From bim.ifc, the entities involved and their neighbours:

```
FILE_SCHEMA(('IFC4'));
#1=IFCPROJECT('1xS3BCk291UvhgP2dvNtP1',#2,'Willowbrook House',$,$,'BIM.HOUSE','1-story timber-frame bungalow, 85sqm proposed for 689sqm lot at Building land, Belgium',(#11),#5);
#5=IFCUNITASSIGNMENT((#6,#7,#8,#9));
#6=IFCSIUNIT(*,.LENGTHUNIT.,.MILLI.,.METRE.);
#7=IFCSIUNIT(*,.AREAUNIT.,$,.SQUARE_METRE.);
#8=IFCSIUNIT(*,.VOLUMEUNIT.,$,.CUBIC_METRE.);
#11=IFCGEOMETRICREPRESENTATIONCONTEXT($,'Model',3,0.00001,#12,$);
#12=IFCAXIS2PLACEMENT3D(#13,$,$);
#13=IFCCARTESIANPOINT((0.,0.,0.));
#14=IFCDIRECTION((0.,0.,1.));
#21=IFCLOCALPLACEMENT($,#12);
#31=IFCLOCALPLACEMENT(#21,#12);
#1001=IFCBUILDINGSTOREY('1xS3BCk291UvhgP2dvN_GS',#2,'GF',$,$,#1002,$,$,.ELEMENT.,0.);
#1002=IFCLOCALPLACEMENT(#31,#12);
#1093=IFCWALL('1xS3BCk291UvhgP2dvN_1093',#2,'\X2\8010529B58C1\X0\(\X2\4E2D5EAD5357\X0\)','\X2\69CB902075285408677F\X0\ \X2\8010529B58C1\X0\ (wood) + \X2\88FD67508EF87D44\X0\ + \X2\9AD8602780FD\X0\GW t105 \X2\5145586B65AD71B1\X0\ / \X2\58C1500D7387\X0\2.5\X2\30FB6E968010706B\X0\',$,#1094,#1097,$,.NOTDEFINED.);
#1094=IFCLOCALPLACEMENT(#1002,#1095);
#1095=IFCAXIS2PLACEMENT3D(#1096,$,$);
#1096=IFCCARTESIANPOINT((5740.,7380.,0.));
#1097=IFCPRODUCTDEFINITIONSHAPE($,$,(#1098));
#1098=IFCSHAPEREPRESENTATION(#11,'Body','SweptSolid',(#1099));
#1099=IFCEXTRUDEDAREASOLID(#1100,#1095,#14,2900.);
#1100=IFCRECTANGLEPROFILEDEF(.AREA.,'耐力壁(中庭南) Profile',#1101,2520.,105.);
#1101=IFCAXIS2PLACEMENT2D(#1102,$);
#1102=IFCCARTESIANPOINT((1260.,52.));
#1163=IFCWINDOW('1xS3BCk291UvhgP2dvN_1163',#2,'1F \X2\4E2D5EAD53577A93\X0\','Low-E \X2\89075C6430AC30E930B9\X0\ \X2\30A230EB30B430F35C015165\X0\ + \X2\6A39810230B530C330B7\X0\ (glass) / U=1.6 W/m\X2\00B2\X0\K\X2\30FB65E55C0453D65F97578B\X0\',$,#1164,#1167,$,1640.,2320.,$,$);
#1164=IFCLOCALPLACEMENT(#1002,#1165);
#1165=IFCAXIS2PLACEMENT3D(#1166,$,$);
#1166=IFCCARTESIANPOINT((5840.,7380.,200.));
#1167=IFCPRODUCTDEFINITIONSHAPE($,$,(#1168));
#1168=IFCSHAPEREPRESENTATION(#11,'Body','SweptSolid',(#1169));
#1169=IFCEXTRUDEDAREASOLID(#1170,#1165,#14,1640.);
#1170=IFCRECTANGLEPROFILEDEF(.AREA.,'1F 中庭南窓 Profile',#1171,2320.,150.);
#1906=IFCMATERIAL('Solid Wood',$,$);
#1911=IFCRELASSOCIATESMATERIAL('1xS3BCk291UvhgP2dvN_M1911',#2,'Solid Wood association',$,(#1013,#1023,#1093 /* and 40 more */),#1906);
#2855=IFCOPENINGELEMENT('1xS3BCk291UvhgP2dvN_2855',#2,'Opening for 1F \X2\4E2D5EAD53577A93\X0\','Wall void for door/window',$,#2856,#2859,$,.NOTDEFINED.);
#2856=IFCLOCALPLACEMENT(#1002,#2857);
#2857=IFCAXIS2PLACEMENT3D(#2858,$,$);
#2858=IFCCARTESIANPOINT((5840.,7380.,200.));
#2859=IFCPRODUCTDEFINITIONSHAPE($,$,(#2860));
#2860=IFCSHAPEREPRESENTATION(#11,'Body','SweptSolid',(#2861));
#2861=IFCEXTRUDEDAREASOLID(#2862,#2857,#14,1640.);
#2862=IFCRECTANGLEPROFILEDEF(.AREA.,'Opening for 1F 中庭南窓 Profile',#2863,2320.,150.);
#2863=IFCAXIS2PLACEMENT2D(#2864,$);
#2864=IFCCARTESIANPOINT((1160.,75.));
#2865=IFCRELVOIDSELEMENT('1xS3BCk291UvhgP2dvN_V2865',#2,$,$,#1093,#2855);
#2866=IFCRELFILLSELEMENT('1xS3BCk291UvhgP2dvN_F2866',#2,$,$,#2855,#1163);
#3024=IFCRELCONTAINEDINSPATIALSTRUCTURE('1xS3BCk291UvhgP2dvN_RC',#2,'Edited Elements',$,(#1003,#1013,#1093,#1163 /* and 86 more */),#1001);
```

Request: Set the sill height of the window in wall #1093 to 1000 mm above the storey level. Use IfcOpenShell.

```python
import numpy as np
import ifcopenshell
import ifcopenshell.api.geometry
import ifcopenshell.geom
import ifcopenshell.util.element
import ifcopenshell.util.placement
import ifcopenshell.util.shape
import ifcopenshell.util.unit

model = ifcopenshell.open("bim.ifc")
unit_scale = ifcopenshell.util.unit.calculate_unit_scale(model)

window = model.by_guid("1xS3BCk291UvhgP2dvN_1163")
opening = window.FillsVoids[0].RelatingOpeningElement
storey = ifcopenshell.util.element.get_container(window, ifc_class="IfcBuildingStorey")
level = ifcopenshell.util.placement.get_local_placement(storey.ObjectPlacement)[2, 3]

# The opening's origin need not be at the sill, so measure its lowest point.
shape = ifcopenshell.geom.create_shape(ifcopenshell.geom.settings(), opening)
bottom = ifcopenshell.util.shape.get_shape_bottom_elevation(shape, shape.geometry) / unit_scale
dz = level + 1 / unit_scale - bottom

shift = np.array([0.0, 0.0, dz])
# The window is not placed relative to its opening, so move both.
for product in (opening, window):
    matrix = ifcopenshell.util.placement.get_local_placement(product.ObjectPlacement)
    matrix[:3, 3] += shift
    ifcopenshell.api.geometry.edit_object_placement(model, product=product, matrix=matrix, is_si=False)

print(f"moved by {dz * unit_scale:+.3f} m")

model.write("bim-out.ifc")
```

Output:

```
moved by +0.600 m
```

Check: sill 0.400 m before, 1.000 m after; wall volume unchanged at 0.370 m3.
